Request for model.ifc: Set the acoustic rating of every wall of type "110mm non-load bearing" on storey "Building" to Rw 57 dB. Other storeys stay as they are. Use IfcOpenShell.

First a look at what the model holds.

```python
import ifcopenshell
import ifcopenshell.util.element

model = ifcopenshell.open("model.ifc")
print(model.schema)
storey = next(s for s in model.by_type("IfcBuildingStorey") if s.Name == "Building")
walls = [e for e in ifcopenshell.util.element.get_decomposition(storey) if e.is_a("IfcWall")]
seen = {}
for e in walls:
    element_type = ifcopenshell.util.element.get_type(e)
    key = (element_type.Name if element_type != e and element_type else None, ifcopenshell.util.element.get_pset(e, "Pset_WallCommon", "AcousticRating"))
    seen[key] = seen.get(key, 0) + 1
for (name, value), count in sorted(seen.items(), key=str):
    print(count, "x", name, "|", value)
```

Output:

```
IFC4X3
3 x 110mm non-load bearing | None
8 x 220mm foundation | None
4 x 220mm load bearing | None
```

```python
import ifcopenshell
import ifcopenshell.api.pset
import ifcopenshell.util.element

model = ifcopenshell.open("model.ifc")

storey = next(s for s in model.by_type("IfcBuildingStorey") if s.Name == "Building")
walls = [e for e in ifcopenshell.util.element.get_decomposition(storey) if e.is_a("IfcWall")]

count = 0
for e in walls:
    element_type = ifcopenshell.util.element.get_type(e)
    if element_type in (None, e) or element_type.Name != "110mm non-load bearing":
        continue
    # add_pset returns the element's existing set when there is one.
    pset = ifcopenshell.api.pset.add_pset(model, product=e, name="Pset_WallCommon")
    ifcopenshell.api.pset.edit_pset(model, pset=pset, properties={"AcousticRating": "Rw 57 dB"})
    count += 1

print(count, "walls updated")

model.write("model_rev.ifc")
```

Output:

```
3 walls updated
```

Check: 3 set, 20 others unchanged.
